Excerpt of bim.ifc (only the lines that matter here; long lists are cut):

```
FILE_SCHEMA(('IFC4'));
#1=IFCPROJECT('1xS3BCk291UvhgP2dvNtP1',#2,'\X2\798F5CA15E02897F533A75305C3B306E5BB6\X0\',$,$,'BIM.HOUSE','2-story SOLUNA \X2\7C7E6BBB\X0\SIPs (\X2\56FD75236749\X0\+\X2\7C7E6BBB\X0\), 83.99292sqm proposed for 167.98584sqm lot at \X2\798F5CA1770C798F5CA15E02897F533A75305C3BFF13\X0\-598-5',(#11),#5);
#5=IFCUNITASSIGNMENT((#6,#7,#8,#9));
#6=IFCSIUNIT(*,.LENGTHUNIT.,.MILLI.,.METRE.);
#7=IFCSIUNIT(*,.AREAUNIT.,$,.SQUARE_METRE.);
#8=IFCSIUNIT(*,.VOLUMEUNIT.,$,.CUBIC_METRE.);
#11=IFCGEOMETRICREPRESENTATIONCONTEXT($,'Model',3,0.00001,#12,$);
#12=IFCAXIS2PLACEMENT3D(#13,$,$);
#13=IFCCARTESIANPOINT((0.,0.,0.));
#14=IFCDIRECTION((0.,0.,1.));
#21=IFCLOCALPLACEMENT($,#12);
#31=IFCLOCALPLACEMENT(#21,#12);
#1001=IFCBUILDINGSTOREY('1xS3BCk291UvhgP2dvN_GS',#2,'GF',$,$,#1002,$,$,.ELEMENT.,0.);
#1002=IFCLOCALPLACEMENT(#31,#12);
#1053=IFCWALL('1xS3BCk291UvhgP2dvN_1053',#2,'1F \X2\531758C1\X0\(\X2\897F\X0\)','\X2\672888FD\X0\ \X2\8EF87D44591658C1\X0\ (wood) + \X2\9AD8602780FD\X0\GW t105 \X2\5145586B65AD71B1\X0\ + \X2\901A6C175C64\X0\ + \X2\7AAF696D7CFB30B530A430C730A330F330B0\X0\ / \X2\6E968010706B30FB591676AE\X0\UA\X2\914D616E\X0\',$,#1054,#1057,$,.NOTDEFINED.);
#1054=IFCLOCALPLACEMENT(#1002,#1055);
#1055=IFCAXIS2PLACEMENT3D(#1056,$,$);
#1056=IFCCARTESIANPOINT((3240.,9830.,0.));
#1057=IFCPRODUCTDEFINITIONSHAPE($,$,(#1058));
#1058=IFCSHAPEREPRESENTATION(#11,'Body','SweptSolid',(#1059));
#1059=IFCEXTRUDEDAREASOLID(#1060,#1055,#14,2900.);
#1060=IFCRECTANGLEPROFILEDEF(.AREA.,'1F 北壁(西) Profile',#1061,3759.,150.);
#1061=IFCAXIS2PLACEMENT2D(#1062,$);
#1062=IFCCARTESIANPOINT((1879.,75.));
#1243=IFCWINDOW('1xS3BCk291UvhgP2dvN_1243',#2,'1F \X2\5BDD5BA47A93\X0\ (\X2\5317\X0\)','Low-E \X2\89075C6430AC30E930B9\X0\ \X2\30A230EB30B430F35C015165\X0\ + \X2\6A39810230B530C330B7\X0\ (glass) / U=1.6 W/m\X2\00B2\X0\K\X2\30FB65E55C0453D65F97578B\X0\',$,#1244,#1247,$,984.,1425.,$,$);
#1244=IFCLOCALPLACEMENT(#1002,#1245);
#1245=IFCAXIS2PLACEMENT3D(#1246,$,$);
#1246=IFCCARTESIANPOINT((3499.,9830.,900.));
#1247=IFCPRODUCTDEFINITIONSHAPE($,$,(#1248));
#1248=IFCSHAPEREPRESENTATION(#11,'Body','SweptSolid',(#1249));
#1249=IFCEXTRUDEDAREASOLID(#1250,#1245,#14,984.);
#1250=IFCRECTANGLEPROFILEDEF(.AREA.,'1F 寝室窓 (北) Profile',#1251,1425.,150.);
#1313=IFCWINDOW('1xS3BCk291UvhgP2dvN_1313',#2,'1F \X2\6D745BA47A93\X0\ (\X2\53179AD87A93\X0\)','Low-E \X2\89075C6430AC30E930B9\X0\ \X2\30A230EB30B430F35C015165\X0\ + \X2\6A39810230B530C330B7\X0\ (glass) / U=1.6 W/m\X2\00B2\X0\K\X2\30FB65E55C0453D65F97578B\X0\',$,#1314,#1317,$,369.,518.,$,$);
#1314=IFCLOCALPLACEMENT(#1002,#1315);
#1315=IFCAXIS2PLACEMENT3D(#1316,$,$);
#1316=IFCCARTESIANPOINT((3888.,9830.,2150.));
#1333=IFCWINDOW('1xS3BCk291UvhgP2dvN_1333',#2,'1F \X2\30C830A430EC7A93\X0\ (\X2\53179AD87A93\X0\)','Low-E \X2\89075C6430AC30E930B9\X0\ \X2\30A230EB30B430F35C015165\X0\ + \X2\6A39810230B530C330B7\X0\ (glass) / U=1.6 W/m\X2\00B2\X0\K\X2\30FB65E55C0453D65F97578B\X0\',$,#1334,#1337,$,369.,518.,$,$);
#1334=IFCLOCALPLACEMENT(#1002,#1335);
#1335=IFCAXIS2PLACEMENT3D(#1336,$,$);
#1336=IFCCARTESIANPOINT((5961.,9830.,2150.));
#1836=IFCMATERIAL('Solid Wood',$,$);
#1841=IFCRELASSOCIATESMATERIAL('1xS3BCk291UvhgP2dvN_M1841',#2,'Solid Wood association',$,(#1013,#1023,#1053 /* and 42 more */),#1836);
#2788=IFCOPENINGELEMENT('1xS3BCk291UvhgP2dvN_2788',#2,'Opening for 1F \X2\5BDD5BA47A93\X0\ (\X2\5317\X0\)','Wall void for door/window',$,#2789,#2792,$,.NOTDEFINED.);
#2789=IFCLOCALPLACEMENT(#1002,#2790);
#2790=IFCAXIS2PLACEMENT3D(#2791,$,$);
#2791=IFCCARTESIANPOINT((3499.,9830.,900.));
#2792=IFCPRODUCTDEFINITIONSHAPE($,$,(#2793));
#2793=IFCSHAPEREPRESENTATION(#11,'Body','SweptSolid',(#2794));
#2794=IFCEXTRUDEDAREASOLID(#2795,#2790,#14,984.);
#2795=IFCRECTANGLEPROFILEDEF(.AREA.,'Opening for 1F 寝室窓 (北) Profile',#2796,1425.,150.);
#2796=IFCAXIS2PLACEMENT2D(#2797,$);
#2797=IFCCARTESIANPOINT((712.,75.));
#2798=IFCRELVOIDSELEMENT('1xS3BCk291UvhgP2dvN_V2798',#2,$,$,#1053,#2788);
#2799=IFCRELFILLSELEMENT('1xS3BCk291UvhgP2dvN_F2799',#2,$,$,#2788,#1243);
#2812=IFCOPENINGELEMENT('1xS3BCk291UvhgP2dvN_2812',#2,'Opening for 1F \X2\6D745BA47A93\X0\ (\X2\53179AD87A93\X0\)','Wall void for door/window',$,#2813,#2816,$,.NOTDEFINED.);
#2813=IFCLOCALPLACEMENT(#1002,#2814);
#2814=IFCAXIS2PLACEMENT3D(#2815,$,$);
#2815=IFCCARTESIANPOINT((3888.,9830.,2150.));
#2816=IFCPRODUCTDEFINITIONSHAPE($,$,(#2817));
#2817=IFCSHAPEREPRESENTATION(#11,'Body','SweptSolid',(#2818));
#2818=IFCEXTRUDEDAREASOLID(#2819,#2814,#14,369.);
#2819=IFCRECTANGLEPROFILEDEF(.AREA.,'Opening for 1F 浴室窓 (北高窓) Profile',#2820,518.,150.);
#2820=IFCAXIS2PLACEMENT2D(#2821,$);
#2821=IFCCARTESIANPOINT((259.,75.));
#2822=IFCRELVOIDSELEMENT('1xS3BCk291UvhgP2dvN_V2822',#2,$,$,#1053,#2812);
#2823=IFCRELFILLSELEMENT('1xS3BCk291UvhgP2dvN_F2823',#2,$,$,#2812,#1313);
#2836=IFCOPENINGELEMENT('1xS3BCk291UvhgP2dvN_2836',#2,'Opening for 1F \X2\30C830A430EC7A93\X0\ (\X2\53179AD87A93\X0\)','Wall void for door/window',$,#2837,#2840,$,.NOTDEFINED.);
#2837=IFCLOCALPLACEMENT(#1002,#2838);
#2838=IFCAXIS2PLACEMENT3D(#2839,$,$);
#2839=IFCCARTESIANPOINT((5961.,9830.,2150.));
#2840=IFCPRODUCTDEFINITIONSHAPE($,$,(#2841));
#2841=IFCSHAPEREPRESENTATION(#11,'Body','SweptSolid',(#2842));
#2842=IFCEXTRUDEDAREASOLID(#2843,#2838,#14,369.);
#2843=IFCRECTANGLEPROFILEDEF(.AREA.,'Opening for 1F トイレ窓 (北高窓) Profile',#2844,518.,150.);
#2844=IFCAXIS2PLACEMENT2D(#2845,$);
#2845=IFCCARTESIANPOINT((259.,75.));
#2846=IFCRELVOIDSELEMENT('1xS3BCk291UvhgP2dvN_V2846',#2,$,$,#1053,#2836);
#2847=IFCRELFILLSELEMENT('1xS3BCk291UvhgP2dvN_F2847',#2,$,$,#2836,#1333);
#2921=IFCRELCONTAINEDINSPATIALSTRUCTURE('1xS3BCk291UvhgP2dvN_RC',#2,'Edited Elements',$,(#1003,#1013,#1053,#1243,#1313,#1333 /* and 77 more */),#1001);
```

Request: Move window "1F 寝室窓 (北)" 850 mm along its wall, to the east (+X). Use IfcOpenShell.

```python
import ifcopenshell
import ifcopenshell.api.geometry
import ifcopenshell.util.placement
import ifcopenshell.util.unit

model = ifcopenshell.open("bim.ifc")
unit_scale = ifcopenshell.util.unit.calculate_unit_scale(model)

window = model.by_id(1243)
opening = window.FillsVoids[0].RelatingOpeningElement
wall = opening.VoidsElements[0].RelatingBuildingElement

wall_matrix = ifcopenshell.util.placement.get_local_placement(wall.ObjectPlacement)
shift = wall_matrix[:3, 0] * 0.85 / unit_scale
before = ifcopenshell.util.placement.get_local_placement(window.ObjectPlacement)[:3, 3].copy()

# The window is not placed relative to its opening, so move both.
for product in (opening, window):
    matrix = ifcopenshell.util.placement.get_local_placement(product.ObjectPlacement)
    matrix[:3, 3] += shift
    ifcopenshell.api.geometry.edit_object_placement(model, product=product, matrix=matrix, is_si=False)

after = ifcopenshell.util.placement.get_local_placement(window.ObjectPlacement)[:3, 3]
print("window moved by", (after - before).round(3) + 0.0)

model.write("bim_edited.ifc")
```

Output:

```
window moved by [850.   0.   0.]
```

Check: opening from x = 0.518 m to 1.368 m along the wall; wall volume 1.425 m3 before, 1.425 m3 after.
